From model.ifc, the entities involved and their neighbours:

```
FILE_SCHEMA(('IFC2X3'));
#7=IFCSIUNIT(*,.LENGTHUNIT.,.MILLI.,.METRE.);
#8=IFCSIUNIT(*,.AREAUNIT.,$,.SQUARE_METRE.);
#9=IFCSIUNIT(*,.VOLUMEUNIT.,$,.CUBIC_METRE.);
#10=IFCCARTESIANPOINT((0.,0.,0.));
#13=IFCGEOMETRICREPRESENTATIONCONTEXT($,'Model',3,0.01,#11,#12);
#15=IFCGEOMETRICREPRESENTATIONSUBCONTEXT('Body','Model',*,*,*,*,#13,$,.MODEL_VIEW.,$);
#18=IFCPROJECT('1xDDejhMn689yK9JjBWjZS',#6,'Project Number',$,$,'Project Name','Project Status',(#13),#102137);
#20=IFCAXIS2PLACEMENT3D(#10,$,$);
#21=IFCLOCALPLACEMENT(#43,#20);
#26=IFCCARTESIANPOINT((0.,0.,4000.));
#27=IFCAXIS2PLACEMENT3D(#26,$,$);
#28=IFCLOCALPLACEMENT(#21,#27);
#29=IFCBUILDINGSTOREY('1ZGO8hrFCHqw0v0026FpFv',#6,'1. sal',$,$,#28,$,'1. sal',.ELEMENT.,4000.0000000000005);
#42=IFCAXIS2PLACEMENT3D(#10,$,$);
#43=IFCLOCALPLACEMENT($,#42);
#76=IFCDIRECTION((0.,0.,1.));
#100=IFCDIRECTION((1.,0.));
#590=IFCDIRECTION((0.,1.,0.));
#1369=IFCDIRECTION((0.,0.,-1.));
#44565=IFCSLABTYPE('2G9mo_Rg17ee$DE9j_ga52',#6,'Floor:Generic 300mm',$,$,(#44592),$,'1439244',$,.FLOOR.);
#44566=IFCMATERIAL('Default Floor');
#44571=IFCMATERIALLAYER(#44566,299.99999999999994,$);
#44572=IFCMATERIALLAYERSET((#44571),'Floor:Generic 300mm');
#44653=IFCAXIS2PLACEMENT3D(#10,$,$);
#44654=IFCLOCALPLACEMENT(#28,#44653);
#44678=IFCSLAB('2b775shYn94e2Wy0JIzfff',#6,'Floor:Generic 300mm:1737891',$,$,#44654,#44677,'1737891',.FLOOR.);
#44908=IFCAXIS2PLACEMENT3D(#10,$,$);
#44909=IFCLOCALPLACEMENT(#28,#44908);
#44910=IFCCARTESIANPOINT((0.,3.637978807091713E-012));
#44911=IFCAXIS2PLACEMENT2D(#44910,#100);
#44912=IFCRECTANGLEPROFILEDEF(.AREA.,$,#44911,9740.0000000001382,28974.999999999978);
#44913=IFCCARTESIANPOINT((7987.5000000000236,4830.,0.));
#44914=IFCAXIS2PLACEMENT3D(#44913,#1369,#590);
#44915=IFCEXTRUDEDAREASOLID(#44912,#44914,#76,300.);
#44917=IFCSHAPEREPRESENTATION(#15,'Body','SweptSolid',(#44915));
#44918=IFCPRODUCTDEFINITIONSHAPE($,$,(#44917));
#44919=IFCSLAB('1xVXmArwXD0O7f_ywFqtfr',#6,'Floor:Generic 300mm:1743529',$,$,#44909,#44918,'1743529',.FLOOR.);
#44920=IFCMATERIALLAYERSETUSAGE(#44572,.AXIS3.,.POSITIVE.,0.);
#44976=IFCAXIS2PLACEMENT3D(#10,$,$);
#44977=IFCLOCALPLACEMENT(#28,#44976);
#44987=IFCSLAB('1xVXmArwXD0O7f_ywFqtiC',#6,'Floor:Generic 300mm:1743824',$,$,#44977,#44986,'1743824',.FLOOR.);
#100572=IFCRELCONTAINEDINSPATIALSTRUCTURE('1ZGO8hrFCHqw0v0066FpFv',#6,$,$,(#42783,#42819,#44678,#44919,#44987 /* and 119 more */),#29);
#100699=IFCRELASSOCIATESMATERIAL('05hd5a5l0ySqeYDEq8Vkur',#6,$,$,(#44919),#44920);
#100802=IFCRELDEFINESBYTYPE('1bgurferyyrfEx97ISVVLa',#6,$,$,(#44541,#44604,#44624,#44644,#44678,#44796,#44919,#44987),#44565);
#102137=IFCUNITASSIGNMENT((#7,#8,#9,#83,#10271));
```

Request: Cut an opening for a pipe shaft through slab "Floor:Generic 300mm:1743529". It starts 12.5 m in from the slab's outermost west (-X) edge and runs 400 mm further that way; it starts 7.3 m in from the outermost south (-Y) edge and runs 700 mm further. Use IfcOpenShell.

```python
import numpy as np
import ifcopenshell
import ifcopenshell.api.feature
import ifcopenshell.api.geometry
import ifcopenshell.api.root
import ifcopenshell.geom
import ifcopenshell.util.placement
import ifcopenshell.util.representation
import ifcopenshell.util.shape
import ifcopenshell.util.unit

model = ifcopenshell.open("model.ifc")
unit_scale = ifcopenshell.util.unit.calculate_unit_scale(model)
settings = ifcopenshell.geom.settings()


def volume(element):
    """Net volume in cubic metres, openings subtracted."""
    shape = ifcopenshell.geom.create_shape(settings, element)
    return ifcopenshell.util.shape.get_volume(shape.geometry)


slab = model.by_guid("1xVXmArwXD0O7f_ywFqtfr")
before = volume(slab)

# Extent in the slab's own axes, in metres. The edges named are its -X and -Y sides.
slab_shape = ifcopenshell.geom.create_shape(settings, slab)
vertices = ifcopenshell.util.shape.get_vertices(slab_shape.geometry)
x_min, y_min, bottom = vertices.min(axis=0)
top = vertices[:, 2].max()

opening = ifcopenshell.api.root.create_entity(model, ifc_class="IfcOpeningElement", name="Pipe shaft opening")
context = ifcopenshell.util.representation.get_context(model, "Model", "Body", "MODEL_VIEW")
width, depth = 0.4, 0.7
outline = [(0.0, 0.0), (width, 0.0), (width, depth), (0.0, depth), (0.0, 0.0)]
# Overshoot both faces by 50 mm so the cut is clean.
shape = ifcopenshell.api.geometry.add_slab_representation(
    model, context=context, depth=top - bottom + 0.1, polyline=outline
)
ifcopenshell.api.geometry.assign_representation(model, product=opening, representation=shape)

matrix = ifcopenshell.util.placement.get_local_placement(slab.ObjectPlacement)
matrix[:, 3] = matrix @ np.append(np.array([x_min + 12.5, y_min + 7.3, bottom - 0.05]) / unit_scale, 1.0)
ifcopenshell.api.geometry.edit_object_placement(model, product=opening, matrix=matrix, is_si=False)
ifcopenshell.api.feature.add_feature(model, feature=opening, element=slab)

after = volume(slab)

print(f"slab volume {before:.3f} -> {after:.3f} m3")

model.write("model_updated.ifc")
```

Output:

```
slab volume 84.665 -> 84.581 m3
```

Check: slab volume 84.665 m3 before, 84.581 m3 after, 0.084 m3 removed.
